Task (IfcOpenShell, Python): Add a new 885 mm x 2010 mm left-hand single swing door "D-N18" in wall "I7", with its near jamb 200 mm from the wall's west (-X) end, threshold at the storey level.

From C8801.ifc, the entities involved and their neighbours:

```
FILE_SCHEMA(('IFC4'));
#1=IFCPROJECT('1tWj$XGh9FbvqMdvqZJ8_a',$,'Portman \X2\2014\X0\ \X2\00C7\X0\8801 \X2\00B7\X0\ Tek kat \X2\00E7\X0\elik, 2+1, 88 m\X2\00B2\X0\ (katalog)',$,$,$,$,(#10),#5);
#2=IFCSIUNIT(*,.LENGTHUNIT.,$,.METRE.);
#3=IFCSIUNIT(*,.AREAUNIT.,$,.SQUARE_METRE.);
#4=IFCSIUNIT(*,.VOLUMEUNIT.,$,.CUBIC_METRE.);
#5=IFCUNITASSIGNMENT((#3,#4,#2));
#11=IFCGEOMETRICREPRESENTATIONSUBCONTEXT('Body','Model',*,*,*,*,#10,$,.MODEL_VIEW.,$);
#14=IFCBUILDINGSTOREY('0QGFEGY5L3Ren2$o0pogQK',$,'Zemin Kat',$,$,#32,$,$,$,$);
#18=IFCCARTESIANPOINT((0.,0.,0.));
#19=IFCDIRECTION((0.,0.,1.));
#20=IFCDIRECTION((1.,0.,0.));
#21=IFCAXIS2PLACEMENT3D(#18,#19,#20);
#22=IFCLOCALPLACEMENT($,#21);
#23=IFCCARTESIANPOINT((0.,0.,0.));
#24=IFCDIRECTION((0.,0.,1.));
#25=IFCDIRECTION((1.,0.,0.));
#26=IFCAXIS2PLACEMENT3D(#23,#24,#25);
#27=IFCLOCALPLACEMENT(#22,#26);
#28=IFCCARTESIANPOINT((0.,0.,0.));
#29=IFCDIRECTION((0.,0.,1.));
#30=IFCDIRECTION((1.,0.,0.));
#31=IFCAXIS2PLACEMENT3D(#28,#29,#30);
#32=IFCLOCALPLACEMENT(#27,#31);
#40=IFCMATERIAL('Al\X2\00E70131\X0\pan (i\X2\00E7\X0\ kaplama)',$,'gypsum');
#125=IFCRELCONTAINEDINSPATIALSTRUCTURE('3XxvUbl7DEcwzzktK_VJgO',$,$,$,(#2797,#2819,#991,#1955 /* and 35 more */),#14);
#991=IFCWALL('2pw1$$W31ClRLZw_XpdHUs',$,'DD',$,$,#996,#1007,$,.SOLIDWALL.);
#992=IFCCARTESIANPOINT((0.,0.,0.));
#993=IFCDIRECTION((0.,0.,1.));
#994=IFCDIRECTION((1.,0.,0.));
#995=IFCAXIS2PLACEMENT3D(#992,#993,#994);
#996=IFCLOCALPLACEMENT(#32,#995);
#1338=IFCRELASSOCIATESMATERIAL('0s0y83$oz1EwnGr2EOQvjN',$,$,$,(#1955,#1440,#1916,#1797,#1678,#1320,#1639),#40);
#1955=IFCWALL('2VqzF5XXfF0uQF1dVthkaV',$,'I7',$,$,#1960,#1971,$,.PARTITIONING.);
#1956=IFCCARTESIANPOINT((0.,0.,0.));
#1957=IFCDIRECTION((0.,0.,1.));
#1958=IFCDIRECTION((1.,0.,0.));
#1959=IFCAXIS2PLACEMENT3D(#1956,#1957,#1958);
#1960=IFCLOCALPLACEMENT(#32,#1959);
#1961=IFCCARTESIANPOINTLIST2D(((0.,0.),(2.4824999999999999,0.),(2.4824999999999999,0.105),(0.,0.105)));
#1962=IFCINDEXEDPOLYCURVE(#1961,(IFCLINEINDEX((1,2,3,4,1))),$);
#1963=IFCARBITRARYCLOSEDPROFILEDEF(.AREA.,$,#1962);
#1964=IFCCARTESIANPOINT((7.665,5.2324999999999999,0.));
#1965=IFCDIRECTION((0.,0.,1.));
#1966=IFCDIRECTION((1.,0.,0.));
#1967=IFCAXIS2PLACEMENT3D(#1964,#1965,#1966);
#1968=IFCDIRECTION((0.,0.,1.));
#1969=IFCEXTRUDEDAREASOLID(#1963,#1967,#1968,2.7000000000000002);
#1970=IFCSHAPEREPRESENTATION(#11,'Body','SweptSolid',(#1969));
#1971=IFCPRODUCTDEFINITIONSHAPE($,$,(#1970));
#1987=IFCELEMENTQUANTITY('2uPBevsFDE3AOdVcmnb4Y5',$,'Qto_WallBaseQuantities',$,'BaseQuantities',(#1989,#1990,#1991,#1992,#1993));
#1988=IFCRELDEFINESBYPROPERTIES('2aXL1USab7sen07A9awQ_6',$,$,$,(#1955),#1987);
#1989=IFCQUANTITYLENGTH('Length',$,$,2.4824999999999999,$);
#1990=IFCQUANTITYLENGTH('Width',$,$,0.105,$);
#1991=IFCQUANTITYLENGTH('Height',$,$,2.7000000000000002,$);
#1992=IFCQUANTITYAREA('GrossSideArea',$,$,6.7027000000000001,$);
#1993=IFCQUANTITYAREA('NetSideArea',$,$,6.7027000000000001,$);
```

```python
import numpy as np
import ifcopenshell
import ifcopenshell.api.feature
import ifcopenshell.api.geometry
import ifcopenshell.api.pset
import ifcopenshell.api.root
import ifcopenshell.api.spatial
import ifcopenshell.geom
import ifcopenshell.util.element
import ifcopenshell.util.placement
import ifcopenshell.util.representation
import ifcopenshell.util.shape
import ifcopenshell.util.unit

model = ifcopenshell.open("C8801.ifc")
unit_scale = ifcopenshell.util.unit.calculate_unit_scale(model)
area_scale = ifcopenshell.util.unit.calculate_unit_scale(model, "AREAUNIT")
settings = ifcopenshell.geom.settings()


def volume(element):
    """Net volume in cubic metres, openings subtracted."""
    shape = ifcopenshell.geom.create_shape(settings, element)
    return ifcopenshell.util.shape.get_volume(shape.geometry)


wall = model.by_guid("2VqzF5XXfF0uQF1dVthkaV")
storey = ifcopenshell.util.element.get_container(wall, ifc_class="IfcBuildingStorey")
context = ifcopenshell.util.representation.get_context(model, "Model", "Body", "MODEL_VIEW")
before = volume(wall)

width, height, from_end, sill = 0.885, 2.01, 0.2, 0.0  # metres

# The wall runs along its own X axis, and the end named is its -X end.
wall_shape = ifcopenshell.geom.create_shape(settings, wall)
x, y, z = ifcopenshell.util.shape.get_vertices(wall_shape.geometry).T
start = x.min() + from_end
face, thickness = float(y.min()), float(y.max() - y.min())
wall_matrix = ifcopenshell.util.placement.get_local_placement(wall.ObjectPlacement)
level = ifcopenshell.util.placement.get_local_placement(storey.ObjectPlacement)[2, 3]


def in_wall(x, y):
    """Placement at x, y metres in the wall's axes, at sill height."""
    matrix = wall_matrix.copy()
    matrix[:, 3] = wall_matrix @ np.array([x / unit_scale, y / unit_scale, 0.0, 1.0])
    matrix[2, 3] = level + sill / unit_scale
    return matrix


# Opening: a box that overshoots both wall faces by 50 mm.
opening = ifcopenshell.api.root.create_entity(model, ifc_class="IfcOpeningElement", predefined_type="OPENING")
box = ifcopenshell.api.geometry.add_wall_representation(
    model, context=context, length=width, height=height, thickness=thickness + 0.1
)
ifcopenshell.api.geometry.assign_representation(model, product=opening, representation=box)
ifcopenshell.api.geometry.edit_object_placement(model, product=opening, matrix=in_wall(start, face - 0.05), is_si=False)
ifcopenshell.api.feature.add_feature(model, feature=opening, element=wall)

door = ifcopenshell.api.root.create_entity(model, ifc_class="IfcDoor", name="D-N18", predefined_type="DOOR")
door.OverallWidth, door.OverallHeight = width / unit_scale, height / unit_scale
door.OperationType = "SINGLE_SWING_LEFT"
body = ifcopenshell.api.geometry.add_door_representation(
    model,
    context=context,
    overall_width=door.OverallWidth,
    overall_height=door.OverallHeight,
    operation_type="SINGLE_SWING_LEFT",
    lining_properties={"LiningDepth": thickness / unit_scale, "ThresholdDepth": thickness / unit_scale},
)
ifcopenshell.api.geometry.assign_representation(model, product=door, representation=body)
ifcopenshell.api.spatial.assign_container(model, products=[door], relating_structure=storey)
ifcopenshell.api.feature.add_filling(model, opening=opening, element=door)

# The lining spans the wall, so the door starts at the wall face.
ifcopenshell.api.geometry.edit_object_placement(model, product=door, matrix=in_wall(start, face), is_si=False)

after = volume(wall)

# Update the wall's stored quantities.
qto = model.by_id(ifcopenshell.util.element.get_pset(wall, "Qto_WallBaseQuantities", should_inherit=False)["id"])
ifcopenshell.api.pset.edit_qto(model, qto=qto, properties={"NetSideArea": after / thickness / area_scale})

print(f"wall volume {before:.3f} -> {after:.3f} m3")

model.write("C8801_edited.ifc")
```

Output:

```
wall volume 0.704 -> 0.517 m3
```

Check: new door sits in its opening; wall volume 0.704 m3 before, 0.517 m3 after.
